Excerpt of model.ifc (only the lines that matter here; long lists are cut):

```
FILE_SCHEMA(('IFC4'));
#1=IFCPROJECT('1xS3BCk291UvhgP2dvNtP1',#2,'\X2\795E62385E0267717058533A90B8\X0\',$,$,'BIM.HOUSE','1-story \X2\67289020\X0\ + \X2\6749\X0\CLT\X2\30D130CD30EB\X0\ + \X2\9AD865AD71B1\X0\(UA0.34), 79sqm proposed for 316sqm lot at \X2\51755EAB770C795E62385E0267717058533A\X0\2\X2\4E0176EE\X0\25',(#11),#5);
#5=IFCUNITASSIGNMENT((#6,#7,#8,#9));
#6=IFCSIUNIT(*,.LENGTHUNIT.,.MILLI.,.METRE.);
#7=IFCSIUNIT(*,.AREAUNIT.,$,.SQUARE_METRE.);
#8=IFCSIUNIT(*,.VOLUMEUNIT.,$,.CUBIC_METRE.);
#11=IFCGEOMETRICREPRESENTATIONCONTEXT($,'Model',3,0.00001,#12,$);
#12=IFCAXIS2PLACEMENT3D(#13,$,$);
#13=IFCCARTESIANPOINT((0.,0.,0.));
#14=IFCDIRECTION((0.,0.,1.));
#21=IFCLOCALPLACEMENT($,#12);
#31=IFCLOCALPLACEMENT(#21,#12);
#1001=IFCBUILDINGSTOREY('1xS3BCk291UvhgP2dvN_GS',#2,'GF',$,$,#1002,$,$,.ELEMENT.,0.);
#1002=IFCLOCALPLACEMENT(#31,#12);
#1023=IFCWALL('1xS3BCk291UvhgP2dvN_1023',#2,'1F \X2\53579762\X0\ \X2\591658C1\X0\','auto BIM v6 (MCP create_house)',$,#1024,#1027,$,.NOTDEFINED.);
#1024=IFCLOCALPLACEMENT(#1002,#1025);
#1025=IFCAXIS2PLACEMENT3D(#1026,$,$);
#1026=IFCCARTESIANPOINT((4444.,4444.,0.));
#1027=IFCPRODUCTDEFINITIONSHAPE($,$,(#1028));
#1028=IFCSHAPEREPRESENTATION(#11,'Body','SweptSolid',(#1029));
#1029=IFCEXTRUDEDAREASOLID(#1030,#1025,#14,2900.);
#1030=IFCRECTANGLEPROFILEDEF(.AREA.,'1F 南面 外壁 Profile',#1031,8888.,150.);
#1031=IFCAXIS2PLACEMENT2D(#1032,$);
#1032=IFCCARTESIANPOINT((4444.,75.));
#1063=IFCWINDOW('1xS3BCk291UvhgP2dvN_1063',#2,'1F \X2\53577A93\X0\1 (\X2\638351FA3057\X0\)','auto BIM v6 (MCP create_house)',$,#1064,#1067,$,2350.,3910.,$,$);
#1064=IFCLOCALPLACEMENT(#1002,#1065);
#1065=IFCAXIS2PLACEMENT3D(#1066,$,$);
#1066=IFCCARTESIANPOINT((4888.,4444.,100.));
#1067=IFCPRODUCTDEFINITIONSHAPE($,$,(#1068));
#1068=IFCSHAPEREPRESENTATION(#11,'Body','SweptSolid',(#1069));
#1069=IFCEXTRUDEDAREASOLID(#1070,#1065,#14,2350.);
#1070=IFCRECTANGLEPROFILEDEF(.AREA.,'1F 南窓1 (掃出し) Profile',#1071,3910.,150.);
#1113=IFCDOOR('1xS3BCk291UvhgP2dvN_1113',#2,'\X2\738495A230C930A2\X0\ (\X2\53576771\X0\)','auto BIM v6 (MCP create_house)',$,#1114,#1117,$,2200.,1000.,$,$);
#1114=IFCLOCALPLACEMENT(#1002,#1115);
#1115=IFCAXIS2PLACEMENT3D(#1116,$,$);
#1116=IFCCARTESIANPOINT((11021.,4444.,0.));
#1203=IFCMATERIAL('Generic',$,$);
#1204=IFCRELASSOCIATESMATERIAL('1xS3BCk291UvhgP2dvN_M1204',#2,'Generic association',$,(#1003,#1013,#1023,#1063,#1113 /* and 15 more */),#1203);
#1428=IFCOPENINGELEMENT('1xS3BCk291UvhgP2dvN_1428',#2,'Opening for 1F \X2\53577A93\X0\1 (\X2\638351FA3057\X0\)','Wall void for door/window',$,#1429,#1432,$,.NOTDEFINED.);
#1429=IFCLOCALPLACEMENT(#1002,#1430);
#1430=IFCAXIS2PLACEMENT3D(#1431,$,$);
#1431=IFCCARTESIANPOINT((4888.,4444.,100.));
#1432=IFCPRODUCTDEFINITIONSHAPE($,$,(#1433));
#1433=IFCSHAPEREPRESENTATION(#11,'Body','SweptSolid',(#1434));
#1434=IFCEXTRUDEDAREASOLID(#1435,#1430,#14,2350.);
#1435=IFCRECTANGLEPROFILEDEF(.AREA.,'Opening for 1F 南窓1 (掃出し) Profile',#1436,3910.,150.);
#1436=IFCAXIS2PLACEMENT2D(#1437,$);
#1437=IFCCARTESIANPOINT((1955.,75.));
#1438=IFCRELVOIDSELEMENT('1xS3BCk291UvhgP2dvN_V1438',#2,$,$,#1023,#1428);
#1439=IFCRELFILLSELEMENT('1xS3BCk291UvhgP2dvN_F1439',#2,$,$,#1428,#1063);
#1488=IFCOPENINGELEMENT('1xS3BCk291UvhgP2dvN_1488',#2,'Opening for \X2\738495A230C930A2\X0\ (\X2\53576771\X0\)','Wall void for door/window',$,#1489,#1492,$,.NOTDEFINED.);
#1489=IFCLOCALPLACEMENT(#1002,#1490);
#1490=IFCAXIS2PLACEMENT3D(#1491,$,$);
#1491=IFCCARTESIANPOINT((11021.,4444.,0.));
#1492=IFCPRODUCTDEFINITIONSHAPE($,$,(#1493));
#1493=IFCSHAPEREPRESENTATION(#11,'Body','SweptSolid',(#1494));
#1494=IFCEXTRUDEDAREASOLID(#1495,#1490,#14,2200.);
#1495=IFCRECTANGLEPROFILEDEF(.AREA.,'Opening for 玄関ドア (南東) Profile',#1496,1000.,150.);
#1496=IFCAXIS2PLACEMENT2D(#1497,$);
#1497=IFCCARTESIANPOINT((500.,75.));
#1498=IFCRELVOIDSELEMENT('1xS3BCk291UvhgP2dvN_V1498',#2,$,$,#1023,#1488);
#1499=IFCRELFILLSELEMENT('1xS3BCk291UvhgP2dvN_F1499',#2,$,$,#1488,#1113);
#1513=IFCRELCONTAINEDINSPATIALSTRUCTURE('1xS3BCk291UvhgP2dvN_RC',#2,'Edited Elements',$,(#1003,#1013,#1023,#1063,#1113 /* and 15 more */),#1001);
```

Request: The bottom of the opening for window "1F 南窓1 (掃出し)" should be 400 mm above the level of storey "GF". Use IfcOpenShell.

```python
import numpy as np
import ifcopenshell
import ifcopenshell.api.geometry
import ifcopenshell.geom
import ifcopenshell.util.element
import ifcopenshell.util.placement
import ifcopenshell.util.shape
import ifcopenshell.util.unit

model = ifcopenshell.open("model.ifc")
unit_scale = ifcopenshell.util.unit.calculate_unit_scale(model)

window = model.by_id(1063)
opening = window.FillsVoids[0].RelatingOpeningElement
storey = ifcopenshell.util.element.get_container(window, ifc_class="IfcBuildingStorey")
level = ifcopenshell.util.placement.get_local_placement(storey.ObjectPlacement)[2, 3]

# The opening's origin need not be at the sill, so measure its lowest point.
shape = ifcopenshell.geom.create_shape(ifcopenshell.geom.settings(), opening)
bottom = ifcopenshell.util.shape.get_shape_bottom_elevation(shape, shape.geometry) / unit_scale
dz = level + 0.4 / unit_scale - bottom

shift = np.array([0.0, 0.0, dz])
# The window is not placed relative to its opening, so move both.
for product in (opening, window):
    matrix = ifcopenshell.util.placement.get_local_placement(product.ObjectPlacement)
    matrix[:3, 3] += shift
    ifcopenshell.api.geometry.edit_object_placement(model, product=product, matrix=matrix, is_si=False)

print(f"moved by {dz * unit_scale:+.3f} m")

model.write("model_edited.ifc")
```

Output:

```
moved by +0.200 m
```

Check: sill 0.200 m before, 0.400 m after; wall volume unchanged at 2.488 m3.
